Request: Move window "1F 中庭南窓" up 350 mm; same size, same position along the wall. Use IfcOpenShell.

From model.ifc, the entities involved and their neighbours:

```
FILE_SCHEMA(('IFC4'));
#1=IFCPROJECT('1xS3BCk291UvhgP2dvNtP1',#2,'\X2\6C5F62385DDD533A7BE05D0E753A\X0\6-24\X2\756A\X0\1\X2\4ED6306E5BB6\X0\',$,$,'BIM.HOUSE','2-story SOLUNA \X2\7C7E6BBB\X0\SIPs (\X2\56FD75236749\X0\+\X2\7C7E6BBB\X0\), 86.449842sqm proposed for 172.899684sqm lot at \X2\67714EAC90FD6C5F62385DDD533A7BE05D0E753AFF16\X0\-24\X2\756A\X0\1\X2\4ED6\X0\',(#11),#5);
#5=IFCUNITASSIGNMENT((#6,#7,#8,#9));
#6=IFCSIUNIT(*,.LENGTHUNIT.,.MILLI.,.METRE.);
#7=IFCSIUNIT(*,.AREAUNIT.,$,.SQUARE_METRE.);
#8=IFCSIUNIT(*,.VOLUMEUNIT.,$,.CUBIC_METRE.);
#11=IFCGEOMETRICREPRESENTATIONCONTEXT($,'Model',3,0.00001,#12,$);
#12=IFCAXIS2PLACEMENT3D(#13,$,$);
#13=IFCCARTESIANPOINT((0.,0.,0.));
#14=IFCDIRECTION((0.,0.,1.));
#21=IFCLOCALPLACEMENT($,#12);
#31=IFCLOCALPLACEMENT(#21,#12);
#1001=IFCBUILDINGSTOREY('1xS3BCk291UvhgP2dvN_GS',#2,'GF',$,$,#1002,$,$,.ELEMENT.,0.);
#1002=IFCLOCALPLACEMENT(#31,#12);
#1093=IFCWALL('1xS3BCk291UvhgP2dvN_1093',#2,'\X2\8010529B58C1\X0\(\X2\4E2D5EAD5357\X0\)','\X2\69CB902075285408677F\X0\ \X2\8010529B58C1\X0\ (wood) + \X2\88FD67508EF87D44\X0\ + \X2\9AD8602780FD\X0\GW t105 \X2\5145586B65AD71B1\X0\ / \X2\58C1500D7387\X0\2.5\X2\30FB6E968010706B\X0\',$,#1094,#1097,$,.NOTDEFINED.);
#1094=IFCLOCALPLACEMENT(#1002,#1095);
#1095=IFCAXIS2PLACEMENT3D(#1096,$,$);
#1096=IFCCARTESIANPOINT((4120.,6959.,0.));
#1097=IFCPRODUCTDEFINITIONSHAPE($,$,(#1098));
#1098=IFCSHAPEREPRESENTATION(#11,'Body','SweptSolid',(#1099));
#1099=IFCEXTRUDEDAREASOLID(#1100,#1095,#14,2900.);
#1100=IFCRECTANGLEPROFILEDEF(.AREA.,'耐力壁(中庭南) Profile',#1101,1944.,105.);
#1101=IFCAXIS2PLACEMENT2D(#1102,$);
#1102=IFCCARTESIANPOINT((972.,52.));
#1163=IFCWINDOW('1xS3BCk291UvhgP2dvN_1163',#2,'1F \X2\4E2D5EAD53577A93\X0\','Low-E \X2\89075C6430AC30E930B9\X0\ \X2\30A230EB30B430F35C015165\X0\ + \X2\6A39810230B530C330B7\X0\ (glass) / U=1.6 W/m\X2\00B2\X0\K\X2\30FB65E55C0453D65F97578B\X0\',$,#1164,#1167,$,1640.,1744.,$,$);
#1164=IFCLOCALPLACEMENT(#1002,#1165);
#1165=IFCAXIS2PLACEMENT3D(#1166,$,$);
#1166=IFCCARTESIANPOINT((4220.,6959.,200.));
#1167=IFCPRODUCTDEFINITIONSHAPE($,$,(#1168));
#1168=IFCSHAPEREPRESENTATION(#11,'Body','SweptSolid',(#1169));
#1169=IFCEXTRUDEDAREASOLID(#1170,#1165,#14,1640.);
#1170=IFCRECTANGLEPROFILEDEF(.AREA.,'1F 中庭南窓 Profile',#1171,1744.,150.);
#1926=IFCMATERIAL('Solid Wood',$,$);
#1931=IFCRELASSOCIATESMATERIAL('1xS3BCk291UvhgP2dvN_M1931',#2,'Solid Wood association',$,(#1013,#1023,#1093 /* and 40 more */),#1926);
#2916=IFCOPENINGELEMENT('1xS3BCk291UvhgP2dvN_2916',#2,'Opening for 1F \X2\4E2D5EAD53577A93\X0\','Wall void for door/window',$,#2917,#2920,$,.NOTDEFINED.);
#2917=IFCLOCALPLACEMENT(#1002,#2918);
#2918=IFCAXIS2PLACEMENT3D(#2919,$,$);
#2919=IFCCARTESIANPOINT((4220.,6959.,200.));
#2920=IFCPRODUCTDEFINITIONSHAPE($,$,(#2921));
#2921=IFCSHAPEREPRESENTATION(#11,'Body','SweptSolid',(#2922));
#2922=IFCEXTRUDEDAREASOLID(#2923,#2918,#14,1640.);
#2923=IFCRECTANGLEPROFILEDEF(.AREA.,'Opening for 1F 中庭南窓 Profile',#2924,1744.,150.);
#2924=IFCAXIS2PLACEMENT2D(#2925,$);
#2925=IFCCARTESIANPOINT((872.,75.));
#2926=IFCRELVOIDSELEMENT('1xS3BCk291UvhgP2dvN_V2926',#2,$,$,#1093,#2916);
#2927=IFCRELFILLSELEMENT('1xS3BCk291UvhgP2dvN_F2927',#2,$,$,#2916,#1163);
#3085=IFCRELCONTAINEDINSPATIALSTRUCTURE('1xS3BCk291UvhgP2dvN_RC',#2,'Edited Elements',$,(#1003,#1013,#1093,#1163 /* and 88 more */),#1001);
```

```python
import numpy as np
import ifcopenshell
import ifcopenshell.api.geometry
import ifcopenshell.util.placement
import ifcopenshell.util.unit

model = ifcopenshell.open("model.ifc")
unit_scale = ifcopenshell.util.unit.calculate_unit_scale(model)

window = model.by_id(1163)
opening = window.FillsVoids[0].RelatingOpeningElement
dz = 0.35 / unit_scale

shift = np.array([0.0, 0.0, dz])
# The window is not placed relative to its opening, so move both.
for product in (opening, window):
    matrix = ifcopenshell.util.placement.get_local_placement(product.ObjectPlacement)
    matrix[:3, 3] += shift
    ifcopenshell.api.geometry.edit_object_placement(model, product=product, matrix=matrix, is_si=False)

print(f"moved by {dz * unit_scale:+.3f} m")

model.write("model_edited.ifc")
```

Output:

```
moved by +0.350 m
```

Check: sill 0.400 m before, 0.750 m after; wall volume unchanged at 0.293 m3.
